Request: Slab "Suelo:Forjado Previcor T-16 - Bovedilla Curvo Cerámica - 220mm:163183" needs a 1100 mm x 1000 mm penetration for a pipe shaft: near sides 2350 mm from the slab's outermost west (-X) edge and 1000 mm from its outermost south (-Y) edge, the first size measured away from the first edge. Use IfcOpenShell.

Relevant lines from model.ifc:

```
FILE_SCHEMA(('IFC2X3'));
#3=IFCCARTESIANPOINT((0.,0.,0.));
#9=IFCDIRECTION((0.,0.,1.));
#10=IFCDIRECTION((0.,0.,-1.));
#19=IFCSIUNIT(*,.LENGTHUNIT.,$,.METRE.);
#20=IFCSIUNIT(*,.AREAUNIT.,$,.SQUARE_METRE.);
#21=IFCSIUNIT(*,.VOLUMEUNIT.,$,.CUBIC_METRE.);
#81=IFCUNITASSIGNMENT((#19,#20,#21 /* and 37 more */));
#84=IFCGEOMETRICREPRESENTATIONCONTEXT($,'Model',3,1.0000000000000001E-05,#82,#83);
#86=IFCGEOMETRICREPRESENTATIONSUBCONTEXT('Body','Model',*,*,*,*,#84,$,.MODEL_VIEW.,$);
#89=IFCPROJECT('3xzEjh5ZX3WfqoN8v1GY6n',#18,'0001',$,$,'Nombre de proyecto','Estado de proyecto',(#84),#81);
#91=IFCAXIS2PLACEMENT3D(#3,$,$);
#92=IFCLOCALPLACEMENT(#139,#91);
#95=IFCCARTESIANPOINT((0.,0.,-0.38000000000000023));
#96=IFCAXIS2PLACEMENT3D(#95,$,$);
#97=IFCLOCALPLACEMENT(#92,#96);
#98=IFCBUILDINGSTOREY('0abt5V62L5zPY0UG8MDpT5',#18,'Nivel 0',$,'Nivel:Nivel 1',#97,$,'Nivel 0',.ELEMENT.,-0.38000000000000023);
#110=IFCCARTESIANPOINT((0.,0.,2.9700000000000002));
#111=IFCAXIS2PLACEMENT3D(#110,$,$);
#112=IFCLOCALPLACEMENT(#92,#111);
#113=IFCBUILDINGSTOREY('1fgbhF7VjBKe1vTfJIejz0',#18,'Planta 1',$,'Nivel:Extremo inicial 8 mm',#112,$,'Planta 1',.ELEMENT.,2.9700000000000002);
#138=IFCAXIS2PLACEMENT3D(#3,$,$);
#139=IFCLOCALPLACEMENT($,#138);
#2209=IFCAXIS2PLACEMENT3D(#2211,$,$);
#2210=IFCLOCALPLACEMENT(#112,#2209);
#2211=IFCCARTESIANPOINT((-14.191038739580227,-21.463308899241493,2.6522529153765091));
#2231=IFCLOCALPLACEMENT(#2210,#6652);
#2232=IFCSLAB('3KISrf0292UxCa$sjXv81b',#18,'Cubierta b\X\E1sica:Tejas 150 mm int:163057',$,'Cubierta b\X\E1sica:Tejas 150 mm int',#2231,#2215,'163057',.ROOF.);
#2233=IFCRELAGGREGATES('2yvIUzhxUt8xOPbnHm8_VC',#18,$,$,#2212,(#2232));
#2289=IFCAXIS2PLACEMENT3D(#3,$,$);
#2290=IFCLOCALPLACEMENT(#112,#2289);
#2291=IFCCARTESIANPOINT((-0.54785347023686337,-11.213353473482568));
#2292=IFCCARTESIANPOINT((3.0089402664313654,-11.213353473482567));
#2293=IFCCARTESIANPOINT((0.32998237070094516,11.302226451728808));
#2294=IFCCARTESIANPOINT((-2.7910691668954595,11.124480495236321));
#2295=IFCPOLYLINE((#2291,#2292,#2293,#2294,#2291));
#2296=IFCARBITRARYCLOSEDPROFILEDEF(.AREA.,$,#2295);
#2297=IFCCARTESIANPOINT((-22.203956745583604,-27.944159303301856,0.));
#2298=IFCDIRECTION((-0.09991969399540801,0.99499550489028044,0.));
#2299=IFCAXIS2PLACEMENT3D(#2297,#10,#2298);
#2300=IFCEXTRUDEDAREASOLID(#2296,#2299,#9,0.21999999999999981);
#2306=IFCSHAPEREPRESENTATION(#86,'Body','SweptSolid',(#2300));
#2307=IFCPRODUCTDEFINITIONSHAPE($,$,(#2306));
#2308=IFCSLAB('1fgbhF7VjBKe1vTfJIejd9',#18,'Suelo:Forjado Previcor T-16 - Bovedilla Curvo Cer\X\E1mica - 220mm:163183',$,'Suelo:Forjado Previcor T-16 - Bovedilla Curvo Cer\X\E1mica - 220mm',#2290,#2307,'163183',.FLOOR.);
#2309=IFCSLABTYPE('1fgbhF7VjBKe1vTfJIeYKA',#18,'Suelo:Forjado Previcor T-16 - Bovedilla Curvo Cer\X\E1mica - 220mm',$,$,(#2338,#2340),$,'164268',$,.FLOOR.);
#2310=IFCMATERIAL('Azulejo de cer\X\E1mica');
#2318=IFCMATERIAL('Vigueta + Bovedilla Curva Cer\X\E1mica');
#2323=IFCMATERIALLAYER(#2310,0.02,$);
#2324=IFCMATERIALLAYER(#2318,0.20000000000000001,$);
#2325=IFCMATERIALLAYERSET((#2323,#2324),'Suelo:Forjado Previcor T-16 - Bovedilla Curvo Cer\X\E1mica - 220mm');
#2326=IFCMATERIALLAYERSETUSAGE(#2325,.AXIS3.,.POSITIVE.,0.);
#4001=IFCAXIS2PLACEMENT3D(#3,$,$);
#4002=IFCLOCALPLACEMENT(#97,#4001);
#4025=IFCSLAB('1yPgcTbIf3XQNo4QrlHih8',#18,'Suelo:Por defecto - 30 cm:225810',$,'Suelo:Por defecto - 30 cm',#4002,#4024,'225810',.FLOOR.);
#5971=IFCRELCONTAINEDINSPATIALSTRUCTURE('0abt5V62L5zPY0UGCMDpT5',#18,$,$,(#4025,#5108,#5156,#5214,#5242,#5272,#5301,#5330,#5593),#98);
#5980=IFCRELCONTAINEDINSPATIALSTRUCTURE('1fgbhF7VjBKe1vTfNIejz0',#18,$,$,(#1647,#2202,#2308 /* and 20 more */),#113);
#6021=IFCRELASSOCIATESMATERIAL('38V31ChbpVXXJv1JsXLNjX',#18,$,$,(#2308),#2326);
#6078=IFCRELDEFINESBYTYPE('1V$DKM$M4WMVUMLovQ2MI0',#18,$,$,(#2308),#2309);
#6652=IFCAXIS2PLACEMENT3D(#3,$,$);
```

```python
import numpy as np
import ifcopenshell
import ifcopenshell.api.feature
import ifcopenshell.api.geometry
import ifcopenshell.api.root
import ifcopenshell.geom
import ifcopenshell.util.placement
import ifcopenshell.util.representation
import ifcopenshell.util.shape
import ifcopenshell.util.unit

model = ifcopenshell.open("model.ifc")
unit_scale = ifcopenshell.util.unit.calculate_unit_scale(model)
settings = ifcopenshell.geom.settings()


def volume(element):
    """Net volume in cubic metres, openings subtracted."""
    shape = ifcopenshell.geom.create_shape(settings, element)
    return ifcopenshell.util.shape.get_volume(shape.geometry)


slab = model.by_guid("1fgbhF7VjBKe1vTfJIejd9")
before = volume(slab)

# Extent in the slab's own axes, in metres. The edges named are its -X and -Y sides.
slab_shape = ifcopenshell.geom.create_shape(settings, slab)
vertices = ifcopenshell.util.shape.get_vertices(slab_shape.geometry)
x_min, y_min, bottom = vertices.min(axis=0)
top = vertices[:, 2].max()

opening = ifcopenshell.api.root.create_entity(model, ifc_class="IfcOpeningElement", name="Pipe shaft opening")
context = ifcopenshell.util.representation.get_context(model, "Model", "Body", "MODEL_VIEW")
width, depth = 1.1, 1
outline = [(0.0, 0.0), (width, 0.0), (width, depth), (0.0, depth), (0.0, 0.0)]
# Overshoot both faces by 50 mm so the cut is clean.
shape = ifcopenshell.api.geometry.add_slab_representation(
    model, context=context, depth=top - bottom + 0.1, polyline=outline
)
ifcopenshell.api.geometry.assign_representation(model, product=opening, representation=shape)

matrix = ifcopenshell.util.placement.get_local_placement(slab.ObjectPlacement)
matrix[:, 3] = matrix @ np.append(np.array([x_min + 2.35, y_min + 1, bottom - 0.05]) / unit_scale, 1.0)
ifcopenshell.api.geometry.edit_object_placement(model, product=opening, matrix=matrix, is_si=False)
ifcopenshell.api.feature.add_feature(model, feature=opening, element=slab)

after = volume(slab)

print(f"slab volume {before:.3f} -> {after:.3f} m3")

model.write("model_updated.ifc")
```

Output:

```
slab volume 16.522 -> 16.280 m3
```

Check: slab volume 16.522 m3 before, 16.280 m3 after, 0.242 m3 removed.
